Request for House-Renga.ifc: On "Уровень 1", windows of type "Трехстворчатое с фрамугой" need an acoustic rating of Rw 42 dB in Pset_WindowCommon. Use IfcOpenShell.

First a look at what the model holds.

```python
import ifcopenshell
import ifcopenshell.util.element

model = ifcopenshell.open("House-Renga.ifc")
print(model.schema)
storey = next(s for s in model.by_type("IfcBuildingStorey") if s.Name == "Уровень 1")
windows = [e for e in ifcopenshell.util.element.get_decomposition(storey) if e.is_a("IfcWindow")]
seen = {}
for e in windows:
    element_type = ifcopenshell.util.element.get_type(e)
    key = (element_type.Name if element_type != e and element_type else None, ifcopenshell.util.element.get_pset(e, "Pset_WindowCommon", "AcousticRating"))
    seen[key] = seen.get(key, 0) + 1
for (name, value), count in sorted(seen.items(), key=str):
    print(count, "x", name, "|", value)
```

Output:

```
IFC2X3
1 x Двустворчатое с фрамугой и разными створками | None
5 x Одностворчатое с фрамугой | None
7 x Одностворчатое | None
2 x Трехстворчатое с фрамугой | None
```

```python
import ifcopenshell
import ifcopenshell.api.pset
import ifcopenshell.util.element

model = ifcopenshell.open("House-Renga.ifc")

storey = next(s for s in model.by_type("IfcBuildingStorey") if s.Name == "Уровень 1")
windows = [e for e in ifcopenshell.util.element.get_decomposition(storey) if e.is_a("IfcWindow")]

count = 0
for e in windows:
    element_type = ifcopenshell.util.element.get_type(e)
    if element_type in (None, e) or element_type.Name != "Трехстворчатое с фрамугой":
        continue
    # add_pset returns the element's existing set when there is one.
    pset = ifcopenshell.api.pset.add_pset(model, product=e, name="Pset_WindowCommon")
    ifcopenshell.api.pset.edit_pset(model, pset=pset, properties={"AcousticRating": "Rw 42 dB"})
    count += 1

print(count, "windows updated")

model.write("House-Renga_edited.ifc")
```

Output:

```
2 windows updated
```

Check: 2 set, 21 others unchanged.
